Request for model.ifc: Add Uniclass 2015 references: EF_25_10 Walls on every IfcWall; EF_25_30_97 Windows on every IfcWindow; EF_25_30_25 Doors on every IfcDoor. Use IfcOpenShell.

First a look at what the model holds.

```python
import ifcopenshell

model = ifcopenshell.open("model.ifc")
print(model.schema)
print("classifications:", [c.Name for c in model.by_type("IfcClassification")])
for ifc_class in ("IfcDoor", "IfcRoof", "IfcStair", "IfcWall", "IfcWindow"):
    print(ifc_class, len(model.by_type(ifc_class)))
```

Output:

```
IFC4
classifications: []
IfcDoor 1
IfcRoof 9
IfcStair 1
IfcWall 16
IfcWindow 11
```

```python
import ifcopenshell
import ifcopenshell.api.classification

model = ifcopenshell.open("model.ifc")

system = ifcopenshell.api.classification.add_classification(model, classification="Uniclass 2015")

codes = {
    "IfcWall": ("EF_25_10", "Walls"),
    "IfcWindow": ("EF_25_30_97", "Windows"),
    "IfcDoor": ("EF_25_30_25", "Doors"),
}
for ifc_class, (code, name) in codes.items():
    products = model.by_type(ifc_class)
    ifcopenshell.api.classification.add_reference(
        model, products=products, classification=system, identification=code, name=name
    )
    print(code, len(products))

model.write("model-out.ifc")
```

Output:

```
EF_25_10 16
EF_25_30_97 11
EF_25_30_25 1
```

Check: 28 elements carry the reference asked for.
